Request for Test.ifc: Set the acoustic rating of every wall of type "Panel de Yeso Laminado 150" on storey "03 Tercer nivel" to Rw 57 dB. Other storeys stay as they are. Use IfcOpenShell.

First a look at what the model holds.

```python
import ifcopenshell
import ifcopenshell.util.element

model = ifcopenshell.open("Test.ifc")
print(model.schema)
storey = next(s for s in model.by_type("IfcBuildingStorey") if s.Name == "03 Tercer nivel")
walls = [e for e in ifcopenshell.util.element.get_decomposition(storey) if e.is_a("IfcWall")]
seen = {}
for e in walls:
    element_type = ifcopenshell.util.element.get_type(e)
    key = (element_type.Name if element_type != e and element_type else None, ifcopenshell.util.element.get_pset(e, "Pset_WallCommon", "AcousticRating"))
    seen[key] = seen.get(key, 0) + 1
for (name, value), count in sorted(seen.items(), key=str):
    print(count, "x", name, "|", value)
```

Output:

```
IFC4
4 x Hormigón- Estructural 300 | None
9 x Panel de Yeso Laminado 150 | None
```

```python
import ifcopenshell
import ifcopenshell.api.pset
import ifcopenshell.util.element

model = ifcopenshell.open("Test.ifc")

storey = next(s for s in model.by_type("IfcBuildingStorey") if s.Name == "03 Tercer nivel")
walls = [e for e in ifcopenshell.util.element.get_decomposition(storey) if e.is_a("IfcWall")]

count = 0
for e in walls:
    element_type = ifcopenshell.util.element.get_type(e)
    if element_type in (None, e) or element_type.Name != "Panel de Yeso Laminado 150":
        continue
    # add_pset returns the element's existing set when there is one.
    pset = ifcopenshell.api.pset.add_pset(model, product=e, name="Pset_WallCommon")
    ifcopenshell.api.pset.edit_pset(model, pset=pset, properties={"AcousticRating": "Rw 57 dB"})
    count += 1

print(count, "walls updated")

model.write("Test_rev.ifc")
```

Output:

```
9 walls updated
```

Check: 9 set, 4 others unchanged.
